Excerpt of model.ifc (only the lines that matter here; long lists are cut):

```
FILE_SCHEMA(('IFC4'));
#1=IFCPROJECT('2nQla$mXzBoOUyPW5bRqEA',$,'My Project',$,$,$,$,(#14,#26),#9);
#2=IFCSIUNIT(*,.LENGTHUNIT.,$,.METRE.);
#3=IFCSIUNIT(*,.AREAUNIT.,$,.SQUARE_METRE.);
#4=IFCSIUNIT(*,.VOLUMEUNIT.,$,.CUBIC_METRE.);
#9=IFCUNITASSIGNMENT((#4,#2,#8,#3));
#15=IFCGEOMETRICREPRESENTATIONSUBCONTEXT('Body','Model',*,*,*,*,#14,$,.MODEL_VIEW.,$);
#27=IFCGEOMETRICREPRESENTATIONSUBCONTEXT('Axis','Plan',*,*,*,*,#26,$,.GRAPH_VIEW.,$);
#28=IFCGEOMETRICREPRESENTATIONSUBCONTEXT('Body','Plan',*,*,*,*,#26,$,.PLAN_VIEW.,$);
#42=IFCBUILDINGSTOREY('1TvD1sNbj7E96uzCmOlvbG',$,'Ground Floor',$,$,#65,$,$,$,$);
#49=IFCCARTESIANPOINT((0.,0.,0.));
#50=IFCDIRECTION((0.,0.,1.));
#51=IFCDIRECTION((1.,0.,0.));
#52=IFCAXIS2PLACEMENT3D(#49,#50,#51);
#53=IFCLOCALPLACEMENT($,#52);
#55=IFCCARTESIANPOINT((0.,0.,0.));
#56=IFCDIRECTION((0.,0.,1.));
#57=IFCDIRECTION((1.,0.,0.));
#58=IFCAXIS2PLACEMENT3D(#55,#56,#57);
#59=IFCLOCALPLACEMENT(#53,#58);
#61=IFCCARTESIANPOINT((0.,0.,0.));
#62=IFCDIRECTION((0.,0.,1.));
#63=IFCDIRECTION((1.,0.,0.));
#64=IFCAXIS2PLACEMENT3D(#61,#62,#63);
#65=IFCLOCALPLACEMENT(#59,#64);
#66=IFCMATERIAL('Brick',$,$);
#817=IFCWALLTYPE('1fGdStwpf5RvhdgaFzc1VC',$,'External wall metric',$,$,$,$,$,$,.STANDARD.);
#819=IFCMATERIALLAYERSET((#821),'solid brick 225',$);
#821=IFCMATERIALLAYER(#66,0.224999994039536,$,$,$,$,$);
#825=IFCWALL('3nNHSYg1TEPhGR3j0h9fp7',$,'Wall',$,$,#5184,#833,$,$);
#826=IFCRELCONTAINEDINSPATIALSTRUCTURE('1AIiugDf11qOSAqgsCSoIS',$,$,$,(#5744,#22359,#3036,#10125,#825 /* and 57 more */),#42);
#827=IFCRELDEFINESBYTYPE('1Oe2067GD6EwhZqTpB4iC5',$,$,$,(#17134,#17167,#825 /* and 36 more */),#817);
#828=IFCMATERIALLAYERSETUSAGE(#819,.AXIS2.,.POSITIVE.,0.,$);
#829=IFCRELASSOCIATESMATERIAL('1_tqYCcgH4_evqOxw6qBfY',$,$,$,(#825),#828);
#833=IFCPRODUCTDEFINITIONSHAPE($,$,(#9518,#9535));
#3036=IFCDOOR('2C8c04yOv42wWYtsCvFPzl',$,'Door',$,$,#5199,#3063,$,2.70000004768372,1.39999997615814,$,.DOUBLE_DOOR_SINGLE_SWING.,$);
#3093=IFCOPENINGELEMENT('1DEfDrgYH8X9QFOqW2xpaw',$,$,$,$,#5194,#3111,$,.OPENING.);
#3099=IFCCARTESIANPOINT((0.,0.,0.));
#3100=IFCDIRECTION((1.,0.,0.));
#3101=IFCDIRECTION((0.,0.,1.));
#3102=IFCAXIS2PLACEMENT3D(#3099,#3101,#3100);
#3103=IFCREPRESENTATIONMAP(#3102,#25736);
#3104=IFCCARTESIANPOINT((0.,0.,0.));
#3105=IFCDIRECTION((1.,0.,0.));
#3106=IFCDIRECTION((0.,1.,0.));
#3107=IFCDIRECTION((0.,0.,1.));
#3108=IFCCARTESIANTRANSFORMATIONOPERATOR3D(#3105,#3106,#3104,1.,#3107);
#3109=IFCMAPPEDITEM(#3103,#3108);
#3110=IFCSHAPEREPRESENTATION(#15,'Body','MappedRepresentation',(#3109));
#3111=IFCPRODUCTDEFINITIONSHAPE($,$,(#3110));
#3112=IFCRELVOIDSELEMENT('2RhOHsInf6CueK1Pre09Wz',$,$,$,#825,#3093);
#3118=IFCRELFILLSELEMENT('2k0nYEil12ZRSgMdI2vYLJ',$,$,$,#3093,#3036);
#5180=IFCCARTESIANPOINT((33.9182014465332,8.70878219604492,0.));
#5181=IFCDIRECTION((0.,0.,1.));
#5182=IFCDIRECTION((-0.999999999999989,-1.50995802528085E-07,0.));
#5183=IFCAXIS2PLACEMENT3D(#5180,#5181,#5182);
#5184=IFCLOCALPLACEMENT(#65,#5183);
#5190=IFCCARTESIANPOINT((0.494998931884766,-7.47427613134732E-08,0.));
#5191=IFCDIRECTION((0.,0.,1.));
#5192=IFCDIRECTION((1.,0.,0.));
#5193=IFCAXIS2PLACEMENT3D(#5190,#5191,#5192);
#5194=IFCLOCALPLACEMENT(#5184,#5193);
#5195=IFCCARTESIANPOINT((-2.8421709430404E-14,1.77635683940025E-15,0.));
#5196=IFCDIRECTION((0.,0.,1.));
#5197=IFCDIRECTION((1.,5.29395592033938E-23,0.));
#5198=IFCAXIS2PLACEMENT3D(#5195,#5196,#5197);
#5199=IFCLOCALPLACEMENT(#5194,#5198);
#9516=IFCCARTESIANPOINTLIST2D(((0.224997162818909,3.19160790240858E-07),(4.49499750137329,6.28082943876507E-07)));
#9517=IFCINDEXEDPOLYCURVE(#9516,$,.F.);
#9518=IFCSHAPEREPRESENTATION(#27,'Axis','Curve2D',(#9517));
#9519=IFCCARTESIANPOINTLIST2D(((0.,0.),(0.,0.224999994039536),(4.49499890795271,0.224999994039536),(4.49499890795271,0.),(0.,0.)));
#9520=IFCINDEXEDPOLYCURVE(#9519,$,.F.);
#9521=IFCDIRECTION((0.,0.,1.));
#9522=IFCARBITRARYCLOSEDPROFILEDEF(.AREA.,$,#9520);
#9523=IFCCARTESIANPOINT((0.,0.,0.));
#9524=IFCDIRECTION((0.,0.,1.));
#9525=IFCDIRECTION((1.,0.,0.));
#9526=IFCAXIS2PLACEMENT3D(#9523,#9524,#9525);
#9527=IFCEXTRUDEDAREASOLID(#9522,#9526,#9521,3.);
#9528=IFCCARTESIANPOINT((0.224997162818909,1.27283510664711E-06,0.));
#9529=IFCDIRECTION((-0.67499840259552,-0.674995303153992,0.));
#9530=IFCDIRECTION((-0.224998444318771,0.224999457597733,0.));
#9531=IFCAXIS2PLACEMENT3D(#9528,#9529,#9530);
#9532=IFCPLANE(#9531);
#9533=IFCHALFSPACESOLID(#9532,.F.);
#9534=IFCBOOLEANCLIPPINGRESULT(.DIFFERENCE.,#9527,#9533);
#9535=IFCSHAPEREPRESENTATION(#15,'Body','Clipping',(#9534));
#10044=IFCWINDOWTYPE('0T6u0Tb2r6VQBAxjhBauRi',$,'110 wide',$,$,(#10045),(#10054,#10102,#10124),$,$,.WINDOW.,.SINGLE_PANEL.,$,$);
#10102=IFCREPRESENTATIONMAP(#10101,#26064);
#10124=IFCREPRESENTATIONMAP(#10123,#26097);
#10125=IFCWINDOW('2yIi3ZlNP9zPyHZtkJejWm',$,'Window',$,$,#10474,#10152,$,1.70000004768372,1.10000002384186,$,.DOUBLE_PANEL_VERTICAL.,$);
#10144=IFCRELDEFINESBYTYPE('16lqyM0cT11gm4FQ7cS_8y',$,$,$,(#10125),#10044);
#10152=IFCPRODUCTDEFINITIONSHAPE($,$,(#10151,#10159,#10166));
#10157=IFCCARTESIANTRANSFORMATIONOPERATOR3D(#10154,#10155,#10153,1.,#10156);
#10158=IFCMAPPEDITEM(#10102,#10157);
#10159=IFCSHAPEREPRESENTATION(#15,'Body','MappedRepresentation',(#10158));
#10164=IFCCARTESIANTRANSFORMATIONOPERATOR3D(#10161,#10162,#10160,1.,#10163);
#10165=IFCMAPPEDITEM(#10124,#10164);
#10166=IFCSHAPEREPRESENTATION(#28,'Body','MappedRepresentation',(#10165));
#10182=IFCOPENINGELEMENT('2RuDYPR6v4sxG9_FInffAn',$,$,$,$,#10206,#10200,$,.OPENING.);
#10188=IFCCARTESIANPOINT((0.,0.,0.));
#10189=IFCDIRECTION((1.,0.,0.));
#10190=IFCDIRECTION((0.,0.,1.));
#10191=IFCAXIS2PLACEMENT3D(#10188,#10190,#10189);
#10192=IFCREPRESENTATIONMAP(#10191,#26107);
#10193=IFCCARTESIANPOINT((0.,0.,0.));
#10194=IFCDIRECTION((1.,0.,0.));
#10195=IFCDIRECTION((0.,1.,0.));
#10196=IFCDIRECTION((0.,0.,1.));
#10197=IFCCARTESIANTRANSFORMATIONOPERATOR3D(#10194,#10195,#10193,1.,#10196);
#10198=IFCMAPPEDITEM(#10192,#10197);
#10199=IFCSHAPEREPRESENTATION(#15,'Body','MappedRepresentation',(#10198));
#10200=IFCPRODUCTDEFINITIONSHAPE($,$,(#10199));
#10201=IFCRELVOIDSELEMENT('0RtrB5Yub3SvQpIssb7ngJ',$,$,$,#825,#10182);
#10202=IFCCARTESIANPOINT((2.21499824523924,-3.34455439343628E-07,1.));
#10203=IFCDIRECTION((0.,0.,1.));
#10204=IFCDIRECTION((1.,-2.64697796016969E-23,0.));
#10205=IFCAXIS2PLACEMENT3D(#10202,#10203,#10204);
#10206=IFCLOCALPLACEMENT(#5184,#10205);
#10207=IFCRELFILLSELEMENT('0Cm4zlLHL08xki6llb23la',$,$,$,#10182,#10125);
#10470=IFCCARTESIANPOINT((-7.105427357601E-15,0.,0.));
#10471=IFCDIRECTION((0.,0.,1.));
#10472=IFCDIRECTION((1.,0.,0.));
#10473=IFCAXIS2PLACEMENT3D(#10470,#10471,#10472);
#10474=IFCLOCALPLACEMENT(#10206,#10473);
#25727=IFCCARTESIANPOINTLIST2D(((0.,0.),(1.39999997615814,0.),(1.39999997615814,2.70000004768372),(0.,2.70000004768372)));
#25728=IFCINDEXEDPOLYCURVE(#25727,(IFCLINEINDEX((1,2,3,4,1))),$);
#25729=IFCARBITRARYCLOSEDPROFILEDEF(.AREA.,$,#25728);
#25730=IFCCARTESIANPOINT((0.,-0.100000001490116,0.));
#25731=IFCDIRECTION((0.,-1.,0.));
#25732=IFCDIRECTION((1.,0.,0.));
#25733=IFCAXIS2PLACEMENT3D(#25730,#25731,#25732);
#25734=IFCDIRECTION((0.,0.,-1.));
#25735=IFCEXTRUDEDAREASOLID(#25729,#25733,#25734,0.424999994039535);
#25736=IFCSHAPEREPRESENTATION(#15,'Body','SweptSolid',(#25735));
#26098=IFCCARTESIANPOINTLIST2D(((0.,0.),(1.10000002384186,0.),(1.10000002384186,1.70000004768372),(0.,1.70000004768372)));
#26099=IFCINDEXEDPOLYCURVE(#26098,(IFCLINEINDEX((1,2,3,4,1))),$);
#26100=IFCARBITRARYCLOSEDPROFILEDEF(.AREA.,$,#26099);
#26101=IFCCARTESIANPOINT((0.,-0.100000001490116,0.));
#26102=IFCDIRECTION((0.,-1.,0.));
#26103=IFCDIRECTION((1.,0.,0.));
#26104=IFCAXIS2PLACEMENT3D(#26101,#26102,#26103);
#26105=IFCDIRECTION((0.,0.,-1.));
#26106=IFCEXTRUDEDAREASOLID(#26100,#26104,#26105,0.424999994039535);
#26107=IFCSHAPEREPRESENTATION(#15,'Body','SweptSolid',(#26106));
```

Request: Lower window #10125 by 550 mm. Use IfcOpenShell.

```python
import numpy as np
import ifcopenshell
import ifcopenshell.api.geometry
import ifcopenshell.util.placement
import ifcopenshell.util.unit

model = ifcopenshell.open("model.ifc")
unit_scale = ifcopenshell.util.unit.calculate_unit_scale(model)

window = model.by_guid("2yIi3ZlNP9zPyHZtkJejWm")
opening = window.FillsVoids[0].RelatingOpeningElement
dz = -0.55 / unit_scale

shift = np.array([0.0, 0.0, dz])
# The window is placed relative to its opening, so it follows when the opening moves.
matrix = ifcopenshell.util.placement.get_local_placement(opening.ObjectPlacement)
matrix[:3, 3] += shift
ifcopenshell.api.geometry.edit_object_placement(
    model, product=opening, matrix=matrix, is_si=False, should_transform_children=True
)

print(f"moved by {dz * unit_scale:+.3f} m")

model.write("model_rev.ifc")
```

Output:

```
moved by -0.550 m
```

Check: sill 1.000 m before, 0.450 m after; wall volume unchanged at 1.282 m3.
